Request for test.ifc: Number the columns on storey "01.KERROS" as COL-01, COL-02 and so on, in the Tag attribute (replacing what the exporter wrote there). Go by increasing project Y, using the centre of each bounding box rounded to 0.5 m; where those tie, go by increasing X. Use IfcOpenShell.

First a look at what the model holds.

```python
import ifcopenshell
import ifcopenshell.util.element
import ifcopenshell.util.placement

model = ifcopenshell.open("test.ifc")
print(model.schema)
storey = next(s for s in model.by_type("IfcBuildingStorey") if s.Name == "01.KERROS")
columns = [e for e in ifcopenshell.util.element.get_decomposition(storey) if e.is_a("IfcColumn")]
for e in sorted(columns, key=lambda e: e.id()):
    origin = ifcopenshell.util.placement.get_local_placement(e.ObjectPlacement)[:3, 3]
    print(e.id(), e.Tag, e.Name, origin.round(2) + 0.0, sep=" | ")
```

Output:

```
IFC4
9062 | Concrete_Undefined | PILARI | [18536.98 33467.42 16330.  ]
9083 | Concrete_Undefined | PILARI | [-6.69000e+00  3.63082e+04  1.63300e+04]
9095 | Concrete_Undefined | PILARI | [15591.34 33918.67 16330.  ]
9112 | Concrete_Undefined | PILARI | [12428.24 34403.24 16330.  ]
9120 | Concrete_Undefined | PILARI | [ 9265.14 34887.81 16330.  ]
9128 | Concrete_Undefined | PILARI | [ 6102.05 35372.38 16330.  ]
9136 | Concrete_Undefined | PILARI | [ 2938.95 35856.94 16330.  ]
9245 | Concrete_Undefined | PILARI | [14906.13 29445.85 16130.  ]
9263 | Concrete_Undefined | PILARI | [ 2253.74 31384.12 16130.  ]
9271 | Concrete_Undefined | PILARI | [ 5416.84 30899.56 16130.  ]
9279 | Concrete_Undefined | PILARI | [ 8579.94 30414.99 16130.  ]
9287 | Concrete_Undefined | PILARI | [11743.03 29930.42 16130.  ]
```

```python
import ifcopenshell
import ifcopenshell.geom
import ifcopenshell.util.element
import ifcopenshell.util.shape

model = ifcopenshell.open("test.ifc")
settings = ifcopenshell.geom.settings()
settings.set("use-world-coords", True)


def centre(element):
    shape = ifcopenshell.geom.create_shape(settings, element)
    return ifcopenshell.util.shape.get_bbox_centroid(shape.geometry)


storey = next(s for s in model.by_type("IfcBuildingStorey") if s.Name == "01.KERROS")
columns = [e for e in ifcopenshell.util.element.get_decomposition(storey) if e.is_a("IfcColumn")]

# Insertion points can sit at a corner or the storey origin, so sort by the geometry (in metres).
centres = {e: centre(e) for e in columns}
columns.sort(key=lambda e: (round(centres[e][1] / 0.5), centres[e][0]))

for i, e in enumerate(columns, start=1):
    number = f"COL-{i:02d}"
    e.Tag = number
    print(e.id(), number)

model.write("test-out.ifc")
```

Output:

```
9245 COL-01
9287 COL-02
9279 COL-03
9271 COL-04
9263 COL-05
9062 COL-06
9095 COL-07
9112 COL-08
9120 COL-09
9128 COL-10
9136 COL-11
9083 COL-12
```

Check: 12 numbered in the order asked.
